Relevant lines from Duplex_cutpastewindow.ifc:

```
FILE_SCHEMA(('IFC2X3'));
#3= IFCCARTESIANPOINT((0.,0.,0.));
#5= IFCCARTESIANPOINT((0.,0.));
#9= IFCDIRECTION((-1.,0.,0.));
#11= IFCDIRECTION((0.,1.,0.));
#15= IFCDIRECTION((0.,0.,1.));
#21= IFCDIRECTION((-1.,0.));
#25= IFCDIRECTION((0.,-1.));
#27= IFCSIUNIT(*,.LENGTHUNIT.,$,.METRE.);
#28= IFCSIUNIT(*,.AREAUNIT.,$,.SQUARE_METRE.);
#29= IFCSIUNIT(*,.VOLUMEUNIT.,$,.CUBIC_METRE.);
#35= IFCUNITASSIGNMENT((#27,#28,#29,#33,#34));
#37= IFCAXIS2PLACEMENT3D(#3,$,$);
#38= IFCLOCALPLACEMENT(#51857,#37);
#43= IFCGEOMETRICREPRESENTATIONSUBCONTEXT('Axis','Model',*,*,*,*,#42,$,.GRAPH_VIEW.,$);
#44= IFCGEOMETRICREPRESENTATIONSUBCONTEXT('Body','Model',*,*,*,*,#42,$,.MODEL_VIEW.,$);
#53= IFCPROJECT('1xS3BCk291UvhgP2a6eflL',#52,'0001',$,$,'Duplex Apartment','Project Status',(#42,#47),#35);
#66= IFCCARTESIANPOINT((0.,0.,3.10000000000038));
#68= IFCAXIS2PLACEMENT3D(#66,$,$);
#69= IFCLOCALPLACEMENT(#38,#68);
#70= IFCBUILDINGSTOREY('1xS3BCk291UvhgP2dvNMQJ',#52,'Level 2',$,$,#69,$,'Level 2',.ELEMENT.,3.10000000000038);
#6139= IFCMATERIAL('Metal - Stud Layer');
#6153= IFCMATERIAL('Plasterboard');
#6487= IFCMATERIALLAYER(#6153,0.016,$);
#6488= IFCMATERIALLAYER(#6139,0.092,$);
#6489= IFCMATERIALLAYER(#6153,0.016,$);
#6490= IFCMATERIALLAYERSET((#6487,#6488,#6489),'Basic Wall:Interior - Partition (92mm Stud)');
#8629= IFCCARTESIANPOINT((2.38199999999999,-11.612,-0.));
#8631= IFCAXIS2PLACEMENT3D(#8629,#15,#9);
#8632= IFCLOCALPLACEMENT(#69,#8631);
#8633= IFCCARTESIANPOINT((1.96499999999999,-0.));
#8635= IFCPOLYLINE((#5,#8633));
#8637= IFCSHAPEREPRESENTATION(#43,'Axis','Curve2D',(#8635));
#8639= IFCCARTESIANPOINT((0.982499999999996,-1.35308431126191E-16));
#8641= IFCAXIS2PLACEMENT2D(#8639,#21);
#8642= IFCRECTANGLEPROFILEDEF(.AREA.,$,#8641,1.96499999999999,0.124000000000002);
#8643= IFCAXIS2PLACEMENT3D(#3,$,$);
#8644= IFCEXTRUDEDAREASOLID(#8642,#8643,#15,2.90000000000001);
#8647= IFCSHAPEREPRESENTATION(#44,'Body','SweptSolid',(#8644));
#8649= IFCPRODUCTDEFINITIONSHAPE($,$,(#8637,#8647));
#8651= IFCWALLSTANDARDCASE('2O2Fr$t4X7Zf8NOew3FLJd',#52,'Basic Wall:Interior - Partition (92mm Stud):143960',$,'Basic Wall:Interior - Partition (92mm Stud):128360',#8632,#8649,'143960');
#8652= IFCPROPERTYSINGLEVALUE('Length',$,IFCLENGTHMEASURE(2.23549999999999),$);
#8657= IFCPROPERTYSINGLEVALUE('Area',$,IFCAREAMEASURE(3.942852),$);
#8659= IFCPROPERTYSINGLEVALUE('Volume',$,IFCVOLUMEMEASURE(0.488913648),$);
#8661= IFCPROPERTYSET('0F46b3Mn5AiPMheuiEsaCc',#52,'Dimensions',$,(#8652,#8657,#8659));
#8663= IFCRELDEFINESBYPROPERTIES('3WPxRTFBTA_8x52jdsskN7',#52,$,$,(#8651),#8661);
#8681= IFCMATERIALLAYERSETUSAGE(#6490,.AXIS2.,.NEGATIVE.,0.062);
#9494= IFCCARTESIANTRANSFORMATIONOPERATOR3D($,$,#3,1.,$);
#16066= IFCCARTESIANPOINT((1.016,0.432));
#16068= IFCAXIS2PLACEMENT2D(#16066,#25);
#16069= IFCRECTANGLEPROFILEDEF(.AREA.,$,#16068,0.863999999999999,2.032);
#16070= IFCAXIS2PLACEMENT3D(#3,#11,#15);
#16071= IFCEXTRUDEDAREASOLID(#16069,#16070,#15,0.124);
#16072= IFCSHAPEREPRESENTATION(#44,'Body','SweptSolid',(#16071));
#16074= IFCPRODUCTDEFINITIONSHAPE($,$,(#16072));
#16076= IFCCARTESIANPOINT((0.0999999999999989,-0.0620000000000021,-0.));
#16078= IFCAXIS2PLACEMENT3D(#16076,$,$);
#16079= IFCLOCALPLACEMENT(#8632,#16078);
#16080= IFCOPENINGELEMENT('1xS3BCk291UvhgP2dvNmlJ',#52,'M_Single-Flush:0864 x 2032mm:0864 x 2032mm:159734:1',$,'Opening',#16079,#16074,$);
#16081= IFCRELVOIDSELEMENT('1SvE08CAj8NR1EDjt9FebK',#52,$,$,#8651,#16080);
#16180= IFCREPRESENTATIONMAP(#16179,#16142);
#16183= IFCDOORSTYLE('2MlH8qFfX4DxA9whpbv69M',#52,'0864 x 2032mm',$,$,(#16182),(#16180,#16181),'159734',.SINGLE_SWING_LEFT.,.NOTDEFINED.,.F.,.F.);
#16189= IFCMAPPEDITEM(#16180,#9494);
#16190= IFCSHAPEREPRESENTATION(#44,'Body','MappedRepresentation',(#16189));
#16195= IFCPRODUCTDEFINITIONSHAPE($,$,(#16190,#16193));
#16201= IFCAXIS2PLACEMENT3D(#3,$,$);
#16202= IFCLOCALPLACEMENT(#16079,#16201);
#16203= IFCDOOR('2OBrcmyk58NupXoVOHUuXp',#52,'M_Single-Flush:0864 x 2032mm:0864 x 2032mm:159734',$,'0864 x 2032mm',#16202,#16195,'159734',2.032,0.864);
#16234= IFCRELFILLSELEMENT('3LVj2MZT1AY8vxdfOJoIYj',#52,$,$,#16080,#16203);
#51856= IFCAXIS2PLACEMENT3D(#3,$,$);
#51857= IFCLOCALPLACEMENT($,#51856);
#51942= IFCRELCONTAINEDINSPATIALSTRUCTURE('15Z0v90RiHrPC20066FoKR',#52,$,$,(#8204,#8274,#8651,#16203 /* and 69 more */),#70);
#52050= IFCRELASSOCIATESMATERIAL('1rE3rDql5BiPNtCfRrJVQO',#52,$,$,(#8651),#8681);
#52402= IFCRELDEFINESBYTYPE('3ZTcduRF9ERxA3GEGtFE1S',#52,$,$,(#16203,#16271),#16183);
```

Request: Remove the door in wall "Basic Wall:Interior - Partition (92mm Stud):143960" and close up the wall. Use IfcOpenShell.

```python
import ifcopenshell
import ifcopenshell.api.feature
import ifcopenshell.api.pset
import ifcopenshell.api.root
import ifcopenshell.geom
import ifcopenshell.util.element
import ifcopenshell.util.shape
import ifcopenshell.util.unit

model = ifcopenshell.open("Duplex_cutpastewindow.ifc")
area_scale = ifcopenshell.util.unit.calculate_unit_scale(model, "AREAUNIT")
volume_scale = ifcopenshell.util.unit.calculate_unit_scale(model, "VOLUMEUNIT")
settings = ifcopenshell.geom.settings()


def volume(element):
    """Net volume in cubic metres, openings subtracted."""
    shape = ifcopenshell.geom.create_shape(settings, element)
    return ifcopenshell.util.shape.get_volume(shape.geometry)


door = model.by_id(16203)
opening = door.FillsVoids[0].RelatingOpeningElement
wall = opening.VoidsElements[0].RelatingBuildingElement
before = volume(wall)

ifcopenshell.api.root.remove_product(model, product=door)
ifcopenshell.api.feature.remove_feature(model, feature=opening)

after = volume(wall)
thickness = 0.124  # wall thickness in metres

# Update the wall's stored quantities.
pset = model.by_id(ifcopenshell.util.element.get_pset(wall, "Dimensions", should_inherit=False)["id"])
ifcopenshell.api.pset.edit_pset(model, pset=pset, properties={
    "Area": model.create_entity("IfcAreaMeasure", after / thickness / area_scale),
    "Volume": model.create_entity("IfcVolumeMeasure", after / volume_scale),
})

print(f"wall volume {before:.3f} -> {after:.3f} m3")

model.write("Duplex_cutpastewindow_rev.ifc")
```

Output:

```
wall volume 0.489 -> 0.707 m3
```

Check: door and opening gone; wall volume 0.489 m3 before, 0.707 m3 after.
